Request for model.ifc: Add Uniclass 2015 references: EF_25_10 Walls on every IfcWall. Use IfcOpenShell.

First a look at what the model holds.

```python
import ifcopenshell

model = ifcopenshell.open("model.ifc")
print(model.schema)
print("classifications:", [c.Name for c in model.by_type("IfcClassification")])
for ifc_class in ("IfcDoor", "IfcRoof", "IfcStair", "IfcWall", "IfcWindow"):
    print(ifc_class, len(model.by_type(ifc_class)))
```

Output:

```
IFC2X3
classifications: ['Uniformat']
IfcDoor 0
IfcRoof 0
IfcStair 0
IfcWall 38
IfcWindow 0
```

```python
import ifcopenshell
import ifcopenshell.api.classification

model = ifcopenshell.open("model.ifc")

# IFC2X3 requires Source and Edition and has no link from the project to the system.
system = model.create_entity("IfcClassification", Source="NBS", Edition="2015", Name="Uniclass 2015")

codes = {
    "IfcWall": ("EF_25_10", "Walls"),
}
for ifc_class, (code, name) in codes.items():
    products = model.by_type(ifc_class)
    ifcopenshell.api.classification.add_reference(
        model, products=products, classification=system, identification=code, name=name
    )
    print(code, len(products))

model.write("model-out.ifc")
```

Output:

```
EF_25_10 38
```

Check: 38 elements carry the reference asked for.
